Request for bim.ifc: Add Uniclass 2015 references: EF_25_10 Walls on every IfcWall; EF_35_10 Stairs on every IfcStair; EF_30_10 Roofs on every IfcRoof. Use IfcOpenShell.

First a look at what the model holds.

```python
import ifcopenshell

model = ifcopenshell.open("bim.ifc")
print(model.schema)
print("classifications:", [c.Name for c in model.by_type("IfcClassification")])
for ifc_class in ("IfcDoor", "IfcRoof", "IfcStair", "IfcWall", "IfcWindow"):
    print(ifc_class, len(model.by_type(ifc_class)))
```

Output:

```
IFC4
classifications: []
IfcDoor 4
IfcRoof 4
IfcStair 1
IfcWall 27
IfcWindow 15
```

```python
import ifcopenshell
import ifcopenshell.api.classification

model = ifcopenshell.open("bim.ifc")

system = ifcopenshell.api.classification.add_classification(model, classification="Uniclass 2015")

codes = {
    "IfcWall": ("EF_25_10", "Walls"),
    "IfcStair": ("EF_35_10", "Stairs"),
    "IfcRoof": ("EF_30_10", "Roofs"),
}
for ifc_class, (code, name) in codes.items():
    products = model.by_type(ifc_class)
    ifcopenshell.api.classification.add_reference(
        model, products=products, classification=system, identification=code, name=name
    )
    print(code, len(products))

model.write("bim_edited.ifc")
```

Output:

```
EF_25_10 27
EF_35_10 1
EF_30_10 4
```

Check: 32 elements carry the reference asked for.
